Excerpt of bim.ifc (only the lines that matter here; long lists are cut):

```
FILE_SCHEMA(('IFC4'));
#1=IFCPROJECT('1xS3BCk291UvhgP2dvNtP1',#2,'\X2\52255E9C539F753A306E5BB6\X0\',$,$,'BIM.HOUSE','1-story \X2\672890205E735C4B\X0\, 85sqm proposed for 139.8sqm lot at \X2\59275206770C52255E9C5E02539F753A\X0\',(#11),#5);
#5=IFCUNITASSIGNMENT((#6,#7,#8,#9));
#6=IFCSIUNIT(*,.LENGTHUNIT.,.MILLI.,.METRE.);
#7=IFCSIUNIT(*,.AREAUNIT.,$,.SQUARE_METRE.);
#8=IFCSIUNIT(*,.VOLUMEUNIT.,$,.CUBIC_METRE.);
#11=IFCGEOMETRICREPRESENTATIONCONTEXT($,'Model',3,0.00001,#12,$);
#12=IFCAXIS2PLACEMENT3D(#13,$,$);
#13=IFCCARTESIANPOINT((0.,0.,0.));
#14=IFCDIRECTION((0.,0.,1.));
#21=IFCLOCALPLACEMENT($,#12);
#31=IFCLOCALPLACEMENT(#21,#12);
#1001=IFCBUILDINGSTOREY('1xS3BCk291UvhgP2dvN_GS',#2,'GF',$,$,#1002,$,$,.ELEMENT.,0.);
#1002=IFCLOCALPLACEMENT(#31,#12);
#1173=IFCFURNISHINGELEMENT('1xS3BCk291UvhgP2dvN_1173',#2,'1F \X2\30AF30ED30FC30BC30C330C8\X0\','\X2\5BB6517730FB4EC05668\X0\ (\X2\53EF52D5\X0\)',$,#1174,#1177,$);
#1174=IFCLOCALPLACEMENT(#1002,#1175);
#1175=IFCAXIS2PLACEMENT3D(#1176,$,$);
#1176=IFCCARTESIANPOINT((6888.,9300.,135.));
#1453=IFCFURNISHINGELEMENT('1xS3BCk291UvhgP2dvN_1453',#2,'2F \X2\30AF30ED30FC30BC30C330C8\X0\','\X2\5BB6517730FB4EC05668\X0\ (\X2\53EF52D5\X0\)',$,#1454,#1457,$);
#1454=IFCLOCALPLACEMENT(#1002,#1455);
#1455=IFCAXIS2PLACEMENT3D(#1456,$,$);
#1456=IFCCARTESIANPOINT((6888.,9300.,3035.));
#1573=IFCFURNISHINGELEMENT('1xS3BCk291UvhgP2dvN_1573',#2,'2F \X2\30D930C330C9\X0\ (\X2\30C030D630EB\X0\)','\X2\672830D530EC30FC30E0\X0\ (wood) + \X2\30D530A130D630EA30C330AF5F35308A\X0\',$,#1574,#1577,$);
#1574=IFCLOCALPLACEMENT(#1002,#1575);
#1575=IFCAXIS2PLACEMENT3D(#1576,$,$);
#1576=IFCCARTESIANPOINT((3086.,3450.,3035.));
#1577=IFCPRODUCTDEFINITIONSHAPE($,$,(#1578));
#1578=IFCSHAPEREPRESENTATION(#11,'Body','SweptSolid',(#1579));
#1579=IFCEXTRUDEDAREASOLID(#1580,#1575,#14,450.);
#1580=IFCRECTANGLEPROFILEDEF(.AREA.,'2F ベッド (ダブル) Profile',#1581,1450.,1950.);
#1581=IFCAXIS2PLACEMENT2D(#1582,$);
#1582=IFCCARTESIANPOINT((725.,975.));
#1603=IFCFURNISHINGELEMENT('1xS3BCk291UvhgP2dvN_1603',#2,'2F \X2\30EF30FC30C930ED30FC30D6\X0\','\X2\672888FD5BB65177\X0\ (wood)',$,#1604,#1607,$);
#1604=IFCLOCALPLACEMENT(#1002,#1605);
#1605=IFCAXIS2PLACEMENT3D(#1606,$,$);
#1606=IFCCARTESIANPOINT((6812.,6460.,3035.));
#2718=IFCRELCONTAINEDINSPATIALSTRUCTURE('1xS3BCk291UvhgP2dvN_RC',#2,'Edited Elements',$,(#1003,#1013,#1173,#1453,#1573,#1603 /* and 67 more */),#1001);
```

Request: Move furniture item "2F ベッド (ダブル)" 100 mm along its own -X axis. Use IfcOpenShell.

```python
import ifcopenshell
import ifcopenshell.api.geometry
import ifcopenshell.util.placement
import ifcopenshell.util.unit

model = ifcopenshell.open("bim.ifc")
unit_scale = ifcopenshell.util.unit.calculate_unit_scale(model)

item = model.by_id(1573)
matrix = ifcopenshell.util.placement.get_local_placement(item.ObjectPlacement)
matrix[:3, 3] -= matrix[:3, 0] * 0.1 / unit_scale
ifcopenshell.api.geometry.edit_object_placement(model, product=item, matrix=matrix, is_si=False)

print(ifcopenshell.util.placement.get_local_placement(item.ObjectPlacement).round(3) + 0.0)

model.write("bim_edited.ifc")
```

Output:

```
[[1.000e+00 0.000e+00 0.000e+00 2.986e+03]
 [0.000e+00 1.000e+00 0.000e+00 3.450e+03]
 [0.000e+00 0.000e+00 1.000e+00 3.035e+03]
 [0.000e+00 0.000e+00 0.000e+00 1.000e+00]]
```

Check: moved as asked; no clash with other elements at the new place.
